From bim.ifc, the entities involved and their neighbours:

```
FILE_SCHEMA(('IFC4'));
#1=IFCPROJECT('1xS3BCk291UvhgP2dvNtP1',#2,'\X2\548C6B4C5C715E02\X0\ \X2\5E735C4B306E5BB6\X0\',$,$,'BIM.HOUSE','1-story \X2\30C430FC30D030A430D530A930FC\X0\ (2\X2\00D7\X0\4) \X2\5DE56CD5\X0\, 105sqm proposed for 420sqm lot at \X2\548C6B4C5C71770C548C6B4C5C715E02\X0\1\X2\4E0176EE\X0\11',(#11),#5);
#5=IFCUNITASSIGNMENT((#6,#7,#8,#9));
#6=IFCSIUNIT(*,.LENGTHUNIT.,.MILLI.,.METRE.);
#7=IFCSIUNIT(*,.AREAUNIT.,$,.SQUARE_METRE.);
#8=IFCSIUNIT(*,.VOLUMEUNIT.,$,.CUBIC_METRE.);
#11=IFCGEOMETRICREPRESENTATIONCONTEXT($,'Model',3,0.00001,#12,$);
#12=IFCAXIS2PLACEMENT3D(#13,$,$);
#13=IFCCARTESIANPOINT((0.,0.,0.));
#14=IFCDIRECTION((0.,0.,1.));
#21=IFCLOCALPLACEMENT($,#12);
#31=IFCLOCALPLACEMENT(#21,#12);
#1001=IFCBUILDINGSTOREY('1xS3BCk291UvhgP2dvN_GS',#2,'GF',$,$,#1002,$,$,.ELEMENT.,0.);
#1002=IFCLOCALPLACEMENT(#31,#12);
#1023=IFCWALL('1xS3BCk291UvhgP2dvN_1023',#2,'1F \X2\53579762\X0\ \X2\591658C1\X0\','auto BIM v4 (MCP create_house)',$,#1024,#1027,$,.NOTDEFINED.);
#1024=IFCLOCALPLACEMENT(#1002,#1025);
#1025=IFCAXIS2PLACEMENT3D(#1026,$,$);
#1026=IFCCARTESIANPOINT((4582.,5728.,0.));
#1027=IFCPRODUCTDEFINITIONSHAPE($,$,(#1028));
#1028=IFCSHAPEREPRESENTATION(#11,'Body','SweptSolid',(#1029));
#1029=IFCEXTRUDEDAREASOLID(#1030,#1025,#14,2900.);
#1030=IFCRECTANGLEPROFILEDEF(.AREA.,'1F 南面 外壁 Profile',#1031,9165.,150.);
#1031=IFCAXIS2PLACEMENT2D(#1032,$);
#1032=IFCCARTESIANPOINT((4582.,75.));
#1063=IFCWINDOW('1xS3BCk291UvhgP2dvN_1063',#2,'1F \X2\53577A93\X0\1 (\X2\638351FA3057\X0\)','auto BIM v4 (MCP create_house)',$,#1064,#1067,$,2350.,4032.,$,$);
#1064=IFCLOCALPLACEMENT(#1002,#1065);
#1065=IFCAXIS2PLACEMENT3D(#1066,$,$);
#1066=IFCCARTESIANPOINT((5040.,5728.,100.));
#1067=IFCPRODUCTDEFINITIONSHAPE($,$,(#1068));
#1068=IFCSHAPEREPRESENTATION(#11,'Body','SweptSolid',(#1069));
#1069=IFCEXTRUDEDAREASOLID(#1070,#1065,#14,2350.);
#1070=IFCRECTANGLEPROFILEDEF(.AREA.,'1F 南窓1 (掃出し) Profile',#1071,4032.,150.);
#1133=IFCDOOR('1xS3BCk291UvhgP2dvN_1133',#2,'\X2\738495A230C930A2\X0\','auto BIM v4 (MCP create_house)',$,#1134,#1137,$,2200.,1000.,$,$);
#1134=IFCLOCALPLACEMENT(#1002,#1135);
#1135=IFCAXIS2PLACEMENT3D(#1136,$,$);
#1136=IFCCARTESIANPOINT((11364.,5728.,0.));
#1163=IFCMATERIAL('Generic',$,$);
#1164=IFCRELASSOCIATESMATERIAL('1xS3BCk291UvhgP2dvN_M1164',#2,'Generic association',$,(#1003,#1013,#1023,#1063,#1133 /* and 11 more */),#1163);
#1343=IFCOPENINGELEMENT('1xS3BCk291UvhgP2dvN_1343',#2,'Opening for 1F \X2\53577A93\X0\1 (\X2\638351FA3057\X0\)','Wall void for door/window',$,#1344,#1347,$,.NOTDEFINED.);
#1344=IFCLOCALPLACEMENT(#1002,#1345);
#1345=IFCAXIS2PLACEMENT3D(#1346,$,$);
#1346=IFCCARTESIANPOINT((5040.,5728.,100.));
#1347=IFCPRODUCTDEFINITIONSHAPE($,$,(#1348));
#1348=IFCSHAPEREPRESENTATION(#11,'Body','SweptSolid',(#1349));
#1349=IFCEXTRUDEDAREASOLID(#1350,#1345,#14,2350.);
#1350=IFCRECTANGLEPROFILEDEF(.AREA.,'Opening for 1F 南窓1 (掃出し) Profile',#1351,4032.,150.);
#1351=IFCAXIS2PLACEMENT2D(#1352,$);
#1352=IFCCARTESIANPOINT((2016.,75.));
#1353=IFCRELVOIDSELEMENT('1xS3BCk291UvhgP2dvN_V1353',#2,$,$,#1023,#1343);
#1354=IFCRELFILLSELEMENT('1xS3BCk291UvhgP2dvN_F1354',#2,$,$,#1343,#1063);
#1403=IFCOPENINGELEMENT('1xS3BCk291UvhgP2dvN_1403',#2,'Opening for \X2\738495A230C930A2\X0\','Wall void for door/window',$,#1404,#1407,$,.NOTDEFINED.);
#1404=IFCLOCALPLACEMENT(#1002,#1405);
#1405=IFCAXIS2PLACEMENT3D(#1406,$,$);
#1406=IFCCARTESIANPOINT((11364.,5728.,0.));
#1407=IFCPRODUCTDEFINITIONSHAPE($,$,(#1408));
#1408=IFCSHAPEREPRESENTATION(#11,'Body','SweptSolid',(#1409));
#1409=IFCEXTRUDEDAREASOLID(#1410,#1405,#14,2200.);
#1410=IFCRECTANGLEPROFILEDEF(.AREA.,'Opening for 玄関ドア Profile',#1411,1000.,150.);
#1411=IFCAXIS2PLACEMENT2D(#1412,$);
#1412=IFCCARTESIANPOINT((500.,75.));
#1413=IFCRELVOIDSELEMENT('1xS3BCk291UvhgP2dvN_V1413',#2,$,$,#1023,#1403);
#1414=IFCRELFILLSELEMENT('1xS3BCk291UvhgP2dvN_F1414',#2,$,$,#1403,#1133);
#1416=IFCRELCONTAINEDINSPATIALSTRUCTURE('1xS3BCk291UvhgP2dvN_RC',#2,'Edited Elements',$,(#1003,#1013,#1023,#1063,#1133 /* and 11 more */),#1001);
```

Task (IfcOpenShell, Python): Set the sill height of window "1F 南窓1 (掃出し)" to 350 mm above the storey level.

```python
import numpy as np
import ifcopenshell
import ifcopenshell.api.geometry
import ifcopenshell.geom
import ifcopenshell.util.element
import ifcopenshell.util.placement
import ifcopenshell.util.shape
import ifcopenshell.util.unit

model = ifcopenshell.open("bim.ifc")
unit_scale = ifcopenshell.util.unit.calculate_unit_scale(model)

window = model.by_guid("1xS3BCk291UvhgP2dvN_1063")
opening = window.FillsVoids[0].RelatingOpeningElement
storey = ifcopenshell.util.element.get_container(window, ifc_class="IfcBuildingStorey")
level = ifcopenshell.util.placement.get_local_placement(storey.ObjectPlacement)[2, 3]

# The opening's origin need not be at the sill, so measure its lowest point.
shape = ifcopenshell.geom.create_shape(ifcopenshell.geom.settings(), opening)
bottom = ifcopenshell.util.shape.get_shape_bottom_elevation(shape, shape.geometry) / unit_scale
dz = level + 350.0 - bottom

shift = np.array([0.0, 0.0, dz])
# The window is not placed relative to its opening, so move both.
for product in (opening, window):
    matrix = ifcopenshell.util.placement.get_local_placement(product.ObjectPlacement)
    matrix[:3, 3] += shift
    ifcopenshell.api.geometry.edit_object_placement(model, product=product, matrix=matrix, is_si=False)

print(f"moved by {dz * unit_scale:+.3f} m")

model.write("bim_updated.ifc")
```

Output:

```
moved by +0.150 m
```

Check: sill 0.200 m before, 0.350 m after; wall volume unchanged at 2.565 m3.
